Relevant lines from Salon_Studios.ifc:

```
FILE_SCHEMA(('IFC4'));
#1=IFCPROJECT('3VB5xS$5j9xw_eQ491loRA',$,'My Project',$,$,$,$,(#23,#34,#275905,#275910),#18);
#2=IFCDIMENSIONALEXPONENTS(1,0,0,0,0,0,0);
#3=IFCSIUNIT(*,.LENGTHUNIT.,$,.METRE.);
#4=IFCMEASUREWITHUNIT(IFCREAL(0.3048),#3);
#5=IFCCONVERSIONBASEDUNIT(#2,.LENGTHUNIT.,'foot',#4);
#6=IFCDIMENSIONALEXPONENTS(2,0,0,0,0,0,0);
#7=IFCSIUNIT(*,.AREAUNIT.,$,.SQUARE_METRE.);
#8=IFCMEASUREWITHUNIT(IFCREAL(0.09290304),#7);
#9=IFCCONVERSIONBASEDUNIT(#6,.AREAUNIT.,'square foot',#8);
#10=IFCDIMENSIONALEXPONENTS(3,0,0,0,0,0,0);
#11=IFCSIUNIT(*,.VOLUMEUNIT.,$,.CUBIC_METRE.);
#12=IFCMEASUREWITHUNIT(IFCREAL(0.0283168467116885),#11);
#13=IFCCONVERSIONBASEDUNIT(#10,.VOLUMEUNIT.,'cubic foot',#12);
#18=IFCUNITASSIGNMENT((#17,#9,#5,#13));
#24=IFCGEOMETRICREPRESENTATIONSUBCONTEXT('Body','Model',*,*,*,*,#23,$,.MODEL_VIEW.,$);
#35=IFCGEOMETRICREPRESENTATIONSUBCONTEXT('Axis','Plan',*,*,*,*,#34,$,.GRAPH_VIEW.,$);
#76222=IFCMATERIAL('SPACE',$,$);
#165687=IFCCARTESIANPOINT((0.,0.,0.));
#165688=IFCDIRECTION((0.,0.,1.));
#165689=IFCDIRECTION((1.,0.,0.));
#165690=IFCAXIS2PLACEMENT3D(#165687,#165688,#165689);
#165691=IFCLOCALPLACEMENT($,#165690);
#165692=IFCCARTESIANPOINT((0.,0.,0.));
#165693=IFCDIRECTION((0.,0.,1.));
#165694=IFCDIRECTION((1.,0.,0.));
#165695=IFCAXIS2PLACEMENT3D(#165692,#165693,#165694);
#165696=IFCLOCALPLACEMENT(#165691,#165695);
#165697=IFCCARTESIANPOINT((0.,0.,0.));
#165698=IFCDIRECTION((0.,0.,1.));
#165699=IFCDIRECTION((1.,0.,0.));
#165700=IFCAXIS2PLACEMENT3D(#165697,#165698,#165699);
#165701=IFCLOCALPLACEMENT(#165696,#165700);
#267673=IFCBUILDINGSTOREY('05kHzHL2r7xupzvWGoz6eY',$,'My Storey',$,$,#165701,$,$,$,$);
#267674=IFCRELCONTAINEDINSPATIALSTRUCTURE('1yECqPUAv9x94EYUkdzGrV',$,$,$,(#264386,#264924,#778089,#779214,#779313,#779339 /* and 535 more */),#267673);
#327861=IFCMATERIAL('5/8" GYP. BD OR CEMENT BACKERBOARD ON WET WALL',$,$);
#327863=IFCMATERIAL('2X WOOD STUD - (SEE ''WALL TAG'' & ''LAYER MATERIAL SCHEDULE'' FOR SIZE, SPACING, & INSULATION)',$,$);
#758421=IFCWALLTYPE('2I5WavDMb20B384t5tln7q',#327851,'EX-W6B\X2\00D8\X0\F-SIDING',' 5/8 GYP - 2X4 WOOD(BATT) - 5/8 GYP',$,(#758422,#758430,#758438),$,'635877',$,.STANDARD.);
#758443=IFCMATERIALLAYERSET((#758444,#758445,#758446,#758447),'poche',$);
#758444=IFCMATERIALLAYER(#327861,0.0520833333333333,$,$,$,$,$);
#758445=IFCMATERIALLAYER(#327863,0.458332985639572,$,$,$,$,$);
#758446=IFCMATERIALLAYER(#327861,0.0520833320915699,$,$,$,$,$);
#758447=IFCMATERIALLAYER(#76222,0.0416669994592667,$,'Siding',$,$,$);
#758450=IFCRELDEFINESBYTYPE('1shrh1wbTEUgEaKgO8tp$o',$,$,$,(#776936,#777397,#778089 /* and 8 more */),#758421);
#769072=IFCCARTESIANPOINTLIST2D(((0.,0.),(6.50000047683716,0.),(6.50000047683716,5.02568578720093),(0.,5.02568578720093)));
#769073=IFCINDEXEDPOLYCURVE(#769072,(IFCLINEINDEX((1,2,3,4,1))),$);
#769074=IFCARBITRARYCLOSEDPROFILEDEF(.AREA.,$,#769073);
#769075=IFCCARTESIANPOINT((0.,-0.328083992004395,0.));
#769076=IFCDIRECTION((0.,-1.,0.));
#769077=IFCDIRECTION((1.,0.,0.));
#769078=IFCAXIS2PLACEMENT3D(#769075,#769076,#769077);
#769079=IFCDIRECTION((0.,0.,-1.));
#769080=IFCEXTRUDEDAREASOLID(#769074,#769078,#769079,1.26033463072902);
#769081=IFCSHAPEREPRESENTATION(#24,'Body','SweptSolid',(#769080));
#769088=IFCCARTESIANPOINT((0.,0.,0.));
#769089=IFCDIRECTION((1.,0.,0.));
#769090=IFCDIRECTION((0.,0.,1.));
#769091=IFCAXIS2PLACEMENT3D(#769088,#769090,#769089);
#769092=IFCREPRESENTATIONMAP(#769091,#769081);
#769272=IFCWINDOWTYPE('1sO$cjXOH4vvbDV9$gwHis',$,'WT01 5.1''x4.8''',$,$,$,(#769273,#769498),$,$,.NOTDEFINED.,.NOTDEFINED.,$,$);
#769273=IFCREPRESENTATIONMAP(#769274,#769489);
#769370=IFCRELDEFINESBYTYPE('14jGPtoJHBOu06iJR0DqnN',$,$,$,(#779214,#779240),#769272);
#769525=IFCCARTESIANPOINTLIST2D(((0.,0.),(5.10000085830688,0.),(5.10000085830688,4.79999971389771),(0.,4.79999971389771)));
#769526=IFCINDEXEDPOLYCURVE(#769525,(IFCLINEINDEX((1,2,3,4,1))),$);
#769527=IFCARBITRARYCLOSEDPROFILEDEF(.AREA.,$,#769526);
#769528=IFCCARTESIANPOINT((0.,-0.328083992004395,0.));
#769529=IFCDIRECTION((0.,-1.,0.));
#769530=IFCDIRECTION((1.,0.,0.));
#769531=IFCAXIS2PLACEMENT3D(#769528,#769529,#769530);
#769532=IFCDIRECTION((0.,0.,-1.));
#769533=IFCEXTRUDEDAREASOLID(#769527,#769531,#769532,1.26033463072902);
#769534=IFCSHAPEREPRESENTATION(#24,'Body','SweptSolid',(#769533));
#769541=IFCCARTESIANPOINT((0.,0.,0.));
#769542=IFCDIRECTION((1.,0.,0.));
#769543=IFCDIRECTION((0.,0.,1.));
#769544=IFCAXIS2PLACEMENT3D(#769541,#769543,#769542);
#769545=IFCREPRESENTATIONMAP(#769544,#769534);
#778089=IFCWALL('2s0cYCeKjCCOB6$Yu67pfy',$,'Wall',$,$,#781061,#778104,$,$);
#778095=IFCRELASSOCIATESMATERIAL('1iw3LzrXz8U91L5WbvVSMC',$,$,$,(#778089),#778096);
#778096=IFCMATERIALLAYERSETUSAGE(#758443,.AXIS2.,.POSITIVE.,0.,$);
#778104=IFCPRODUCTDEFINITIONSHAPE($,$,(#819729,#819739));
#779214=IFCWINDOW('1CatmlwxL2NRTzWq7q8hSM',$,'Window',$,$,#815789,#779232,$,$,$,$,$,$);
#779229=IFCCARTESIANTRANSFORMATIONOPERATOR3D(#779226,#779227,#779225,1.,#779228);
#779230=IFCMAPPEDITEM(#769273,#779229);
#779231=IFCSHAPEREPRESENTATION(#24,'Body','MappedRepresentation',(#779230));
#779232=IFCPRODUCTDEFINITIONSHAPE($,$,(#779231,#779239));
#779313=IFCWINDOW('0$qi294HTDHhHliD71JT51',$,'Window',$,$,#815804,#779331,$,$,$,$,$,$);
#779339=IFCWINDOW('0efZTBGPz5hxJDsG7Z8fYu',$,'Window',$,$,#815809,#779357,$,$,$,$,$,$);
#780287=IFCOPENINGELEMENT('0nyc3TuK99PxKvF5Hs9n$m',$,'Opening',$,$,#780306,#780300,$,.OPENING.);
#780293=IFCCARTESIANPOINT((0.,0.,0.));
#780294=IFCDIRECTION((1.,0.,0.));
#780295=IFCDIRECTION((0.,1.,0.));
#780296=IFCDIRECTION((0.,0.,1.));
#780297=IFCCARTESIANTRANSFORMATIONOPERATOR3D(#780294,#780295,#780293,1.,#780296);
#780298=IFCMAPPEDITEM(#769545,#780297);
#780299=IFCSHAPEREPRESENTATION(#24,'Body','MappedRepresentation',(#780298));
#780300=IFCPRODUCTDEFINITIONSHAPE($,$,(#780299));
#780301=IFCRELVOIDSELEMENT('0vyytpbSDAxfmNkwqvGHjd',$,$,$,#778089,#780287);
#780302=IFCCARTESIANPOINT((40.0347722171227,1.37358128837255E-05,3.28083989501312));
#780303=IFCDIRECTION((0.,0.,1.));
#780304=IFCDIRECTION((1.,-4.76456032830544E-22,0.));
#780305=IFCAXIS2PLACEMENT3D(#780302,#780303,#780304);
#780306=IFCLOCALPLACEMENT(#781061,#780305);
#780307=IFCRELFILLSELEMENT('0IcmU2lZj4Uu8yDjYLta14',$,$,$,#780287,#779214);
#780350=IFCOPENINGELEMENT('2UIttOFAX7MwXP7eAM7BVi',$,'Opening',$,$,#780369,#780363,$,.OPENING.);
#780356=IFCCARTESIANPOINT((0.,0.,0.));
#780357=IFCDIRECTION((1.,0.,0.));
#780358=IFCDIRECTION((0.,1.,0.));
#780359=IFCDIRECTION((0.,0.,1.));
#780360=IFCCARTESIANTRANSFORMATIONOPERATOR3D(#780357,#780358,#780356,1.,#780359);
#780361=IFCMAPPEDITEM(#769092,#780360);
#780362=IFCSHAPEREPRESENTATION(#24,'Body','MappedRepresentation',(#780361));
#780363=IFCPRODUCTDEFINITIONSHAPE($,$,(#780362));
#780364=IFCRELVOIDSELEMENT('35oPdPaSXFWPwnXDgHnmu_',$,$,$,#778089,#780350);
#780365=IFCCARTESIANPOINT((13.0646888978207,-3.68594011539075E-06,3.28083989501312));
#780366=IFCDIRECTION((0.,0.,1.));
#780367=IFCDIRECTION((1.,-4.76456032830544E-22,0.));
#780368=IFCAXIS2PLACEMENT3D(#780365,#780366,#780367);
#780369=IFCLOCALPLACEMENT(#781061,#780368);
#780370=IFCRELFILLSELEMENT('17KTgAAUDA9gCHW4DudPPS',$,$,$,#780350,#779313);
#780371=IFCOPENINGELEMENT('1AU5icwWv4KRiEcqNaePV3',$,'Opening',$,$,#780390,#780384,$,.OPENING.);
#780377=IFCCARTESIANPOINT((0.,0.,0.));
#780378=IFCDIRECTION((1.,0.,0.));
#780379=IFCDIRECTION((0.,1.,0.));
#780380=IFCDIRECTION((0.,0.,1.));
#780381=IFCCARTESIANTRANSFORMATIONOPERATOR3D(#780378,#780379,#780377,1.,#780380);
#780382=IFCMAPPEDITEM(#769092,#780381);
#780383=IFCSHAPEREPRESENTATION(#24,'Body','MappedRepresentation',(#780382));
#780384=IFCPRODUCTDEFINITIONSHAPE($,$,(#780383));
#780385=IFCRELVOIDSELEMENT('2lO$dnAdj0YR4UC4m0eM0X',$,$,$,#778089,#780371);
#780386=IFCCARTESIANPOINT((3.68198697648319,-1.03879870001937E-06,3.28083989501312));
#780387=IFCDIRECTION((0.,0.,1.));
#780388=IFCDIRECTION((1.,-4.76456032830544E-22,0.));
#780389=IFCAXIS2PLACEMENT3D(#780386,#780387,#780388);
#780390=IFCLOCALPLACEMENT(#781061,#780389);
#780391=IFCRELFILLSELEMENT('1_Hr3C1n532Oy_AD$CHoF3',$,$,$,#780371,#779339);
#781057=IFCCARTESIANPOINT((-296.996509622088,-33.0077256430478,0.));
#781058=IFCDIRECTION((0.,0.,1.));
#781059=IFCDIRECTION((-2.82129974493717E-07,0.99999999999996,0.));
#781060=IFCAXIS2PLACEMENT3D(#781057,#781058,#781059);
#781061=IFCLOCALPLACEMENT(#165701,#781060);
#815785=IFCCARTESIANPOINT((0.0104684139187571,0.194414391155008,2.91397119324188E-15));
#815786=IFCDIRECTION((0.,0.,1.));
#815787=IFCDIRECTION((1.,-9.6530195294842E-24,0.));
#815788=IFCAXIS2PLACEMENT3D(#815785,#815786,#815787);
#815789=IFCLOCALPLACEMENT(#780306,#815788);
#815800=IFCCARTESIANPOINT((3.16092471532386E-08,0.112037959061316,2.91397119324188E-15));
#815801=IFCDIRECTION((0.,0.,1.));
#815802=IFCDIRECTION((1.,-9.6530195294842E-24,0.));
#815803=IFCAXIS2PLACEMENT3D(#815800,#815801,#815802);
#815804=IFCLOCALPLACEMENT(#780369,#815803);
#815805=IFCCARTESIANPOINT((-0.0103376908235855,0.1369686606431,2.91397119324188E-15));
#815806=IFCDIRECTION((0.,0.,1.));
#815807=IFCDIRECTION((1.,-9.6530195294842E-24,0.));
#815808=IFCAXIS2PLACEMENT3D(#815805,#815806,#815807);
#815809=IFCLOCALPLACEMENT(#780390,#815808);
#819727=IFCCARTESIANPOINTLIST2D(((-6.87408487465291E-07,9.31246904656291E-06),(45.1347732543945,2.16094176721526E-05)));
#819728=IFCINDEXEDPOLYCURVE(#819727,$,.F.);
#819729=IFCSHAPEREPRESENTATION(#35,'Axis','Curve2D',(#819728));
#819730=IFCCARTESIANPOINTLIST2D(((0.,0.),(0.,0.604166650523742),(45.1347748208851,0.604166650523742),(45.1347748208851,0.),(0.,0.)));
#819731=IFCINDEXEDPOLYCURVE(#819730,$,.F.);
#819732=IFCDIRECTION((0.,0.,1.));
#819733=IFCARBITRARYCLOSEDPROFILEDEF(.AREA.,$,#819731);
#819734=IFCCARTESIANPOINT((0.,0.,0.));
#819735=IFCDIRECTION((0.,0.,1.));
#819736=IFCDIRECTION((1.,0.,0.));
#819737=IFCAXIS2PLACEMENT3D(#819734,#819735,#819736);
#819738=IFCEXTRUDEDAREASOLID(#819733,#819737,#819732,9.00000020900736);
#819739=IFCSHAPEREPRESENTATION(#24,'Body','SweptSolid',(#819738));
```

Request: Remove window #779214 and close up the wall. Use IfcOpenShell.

```python
import ifcopenshell
import ifcopenshell.api.feature
import ifcopenshell.api.root
import ifcopenshell.geom
import ifcopenshell.util.shape

model = ifcopenshell.open("Salon_Studios.ifc")
settings = ifcopenshell.geom.settings()


def volume(element):
    """Net volume in cubic metres, openings subtracted."""
    shape = ifcopenshell.geom.create_shape(settings, element)
    return ifcopenshell.util.shape.get_volume(shape.geometry)


window = model.by_guid("1CatmlwxL2NRTzWq7q8hSM")
opening = window.FillsVoids[0].RelatingOpeningElement
wall = opening.VoidsElements[0].RelatingBuildingElement
before = volume(wall)

ifcopenshell.api.root.remove_product(model, product=window)
ifcopenshell.api.feature.remove_feature(model, feature=opening)

after = volume(wall)

print(f"wall volume {before:.3f} -> {after:.3f} m3")

model.write("Salon_Studios_rev.ifc")
```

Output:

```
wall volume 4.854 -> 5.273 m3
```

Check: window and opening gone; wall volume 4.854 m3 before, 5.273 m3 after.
